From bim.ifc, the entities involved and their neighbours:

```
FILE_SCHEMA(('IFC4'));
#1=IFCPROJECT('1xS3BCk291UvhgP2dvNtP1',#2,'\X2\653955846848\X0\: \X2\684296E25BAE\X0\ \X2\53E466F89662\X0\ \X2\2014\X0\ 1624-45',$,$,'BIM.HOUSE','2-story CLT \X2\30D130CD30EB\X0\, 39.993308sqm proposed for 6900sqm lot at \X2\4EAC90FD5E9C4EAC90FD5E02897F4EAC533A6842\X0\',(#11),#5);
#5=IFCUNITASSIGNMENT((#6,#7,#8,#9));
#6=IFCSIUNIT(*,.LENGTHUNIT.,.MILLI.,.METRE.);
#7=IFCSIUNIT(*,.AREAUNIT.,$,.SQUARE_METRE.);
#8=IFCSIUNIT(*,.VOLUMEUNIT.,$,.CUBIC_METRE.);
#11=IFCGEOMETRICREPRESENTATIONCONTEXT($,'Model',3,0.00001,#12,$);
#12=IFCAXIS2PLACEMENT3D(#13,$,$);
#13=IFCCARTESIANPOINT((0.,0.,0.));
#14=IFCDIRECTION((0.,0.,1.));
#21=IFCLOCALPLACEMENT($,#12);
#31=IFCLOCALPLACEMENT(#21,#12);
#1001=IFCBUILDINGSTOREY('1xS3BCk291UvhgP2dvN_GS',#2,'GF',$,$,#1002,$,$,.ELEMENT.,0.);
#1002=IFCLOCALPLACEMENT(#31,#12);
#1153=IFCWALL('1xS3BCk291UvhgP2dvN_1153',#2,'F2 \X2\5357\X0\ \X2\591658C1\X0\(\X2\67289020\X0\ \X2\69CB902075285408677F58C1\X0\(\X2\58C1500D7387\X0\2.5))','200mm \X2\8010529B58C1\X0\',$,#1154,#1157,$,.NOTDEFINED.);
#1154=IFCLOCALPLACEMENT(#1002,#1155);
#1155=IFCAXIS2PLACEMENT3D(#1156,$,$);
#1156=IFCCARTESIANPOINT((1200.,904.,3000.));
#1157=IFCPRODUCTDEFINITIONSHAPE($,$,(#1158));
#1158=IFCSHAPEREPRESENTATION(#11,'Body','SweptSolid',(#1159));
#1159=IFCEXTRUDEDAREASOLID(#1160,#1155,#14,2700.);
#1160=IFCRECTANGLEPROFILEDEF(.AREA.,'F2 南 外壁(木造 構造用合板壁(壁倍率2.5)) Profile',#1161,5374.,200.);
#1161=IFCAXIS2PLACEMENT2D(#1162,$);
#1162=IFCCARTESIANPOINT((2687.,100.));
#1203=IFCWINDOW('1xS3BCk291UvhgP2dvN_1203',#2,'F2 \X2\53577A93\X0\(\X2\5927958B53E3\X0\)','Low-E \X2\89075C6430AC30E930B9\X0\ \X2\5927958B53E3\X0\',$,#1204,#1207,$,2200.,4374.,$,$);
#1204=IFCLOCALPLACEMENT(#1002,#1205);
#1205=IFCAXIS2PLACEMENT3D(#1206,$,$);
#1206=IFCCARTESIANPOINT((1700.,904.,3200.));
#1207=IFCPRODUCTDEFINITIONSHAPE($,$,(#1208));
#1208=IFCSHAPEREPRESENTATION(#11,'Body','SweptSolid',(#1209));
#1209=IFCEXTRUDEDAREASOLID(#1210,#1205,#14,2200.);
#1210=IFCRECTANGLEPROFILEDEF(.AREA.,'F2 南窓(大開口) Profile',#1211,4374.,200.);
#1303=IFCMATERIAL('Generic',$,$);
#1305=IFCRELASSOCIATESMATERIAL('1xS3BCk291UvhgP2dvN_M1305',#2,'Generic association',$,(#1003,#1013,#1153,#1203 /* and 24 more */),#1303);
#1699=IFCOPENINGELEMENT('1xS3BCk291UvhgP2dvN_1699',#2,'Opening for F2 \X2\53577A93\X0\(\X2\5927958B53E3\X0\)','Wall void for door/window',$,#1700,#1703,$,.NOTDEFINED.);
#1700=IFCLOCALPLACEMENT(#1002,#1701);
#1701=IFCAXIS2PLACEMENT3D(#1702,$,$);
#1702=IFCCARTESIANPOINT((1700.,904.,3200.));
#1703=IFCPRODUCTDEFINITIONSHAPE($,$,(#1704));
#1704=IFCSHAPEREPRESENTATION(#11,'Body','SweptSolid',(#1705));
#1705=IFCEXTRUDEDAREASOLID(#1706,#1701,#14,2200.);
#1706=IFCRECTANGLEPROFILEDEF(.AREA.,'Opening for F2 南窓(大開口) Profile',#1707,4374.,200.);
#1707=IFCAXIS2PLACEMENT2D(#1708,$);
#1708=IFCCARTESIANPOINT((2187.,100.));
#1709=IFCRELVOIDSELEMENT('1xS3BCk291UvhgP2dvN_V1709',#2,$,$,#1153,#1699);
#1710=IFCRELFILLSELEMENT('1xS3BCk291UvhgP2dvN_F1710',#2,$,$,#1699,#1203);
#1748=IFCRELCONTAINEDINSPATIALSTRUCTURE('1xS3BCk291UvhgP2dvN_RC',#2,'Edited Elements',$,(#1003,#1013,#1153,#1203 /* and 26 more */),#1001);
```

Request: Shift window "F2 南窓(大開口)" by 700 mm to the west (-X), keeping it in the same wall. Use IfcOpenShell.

```python
import ifcopenshell
import ifcopenshell.api.geometry
import ifcopenshell.util.placement
import ifcopenshell.util.unit

model = ifcopenshell.open("bim.ifc")
unit_scale = ifcopenshell.util.unit.calculate_unit_scale(model)

window = model.by_guid("1xS3BCk291UvhgP2dvN_1203")
opening = window.FillsVoids[0].RelatingOpeningElement
wall = opening.VoidsElements[0].RelatingBuildingElement

wall_matrix = ifcopenshell.util.placement.get_local_placement(wall.ObjectPlacement)
shift = wall_matrix[:3, 0] * -0.7 / unit_scale
before = ifcopenshell.util.placement.get_local_placement(window.ObjectPlacement)[:3, 3].copy()

# The window is not placed relative to its opening, so move both.
for product in (opening, window):
    matrix = ifcopenshell.util.placement.get_local_placement(product.ObjectPlacement)
    matrix[:3, 3] += shift
    ifcopenshell.api.geometry.edit_object_placement(model, product=product, matrix=matrix, is_si=False)

after = ifcopenshell.util.placement.get_local_placement(window.ObjectPlacement)[:3, 3]
print("window moved by", (after - before).round(3) + 0.0)

model.write("bim_edited.ifc")
```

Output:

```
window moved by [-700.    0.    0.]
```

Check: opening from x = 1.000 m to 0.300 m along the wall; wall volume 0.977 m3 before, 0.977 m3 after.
